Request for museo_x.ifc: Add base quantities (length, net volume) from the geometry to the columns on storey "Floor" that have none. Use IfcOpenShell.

First a look at what the model holds.

```python
import ifcopenshell
import ifcopenshell.util.element
import ifcopenshell.util.unit

model = ifcopenshell.open("museo_x.ifc")
print(model.schema)
for unit_type in ("LENGTHUNIT", "AREAUNIT", "VOLUMEUNIT"):
    print(unit_type, ifcopenshell.util.unit.calculate_unit_scale(model, unit_type))
storey = next(s for s in model.by_type("IfcBuildingStorey") if s.Name == "Floor")
columns = [e for e in ifcopenshell.util.element.get_decomposition(storey) if e.is_a("IfcColumn")]
for e in sorted(columns, key=lambda e: e.id()):
    print(e.id(), e.is_a(), e.Name, list(ifcopenshell.util.element.get_psets(e, qtos_only=True)), sep=" | ")
```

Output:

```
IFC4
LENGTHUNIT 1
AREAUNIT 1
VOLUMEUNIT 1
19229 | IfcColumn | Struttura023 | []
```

```python
import ifcopenshell
import ifcopenshell.api.pset
import ifcopenshell.geom
import ifcopenshell.util.element
import ifcopenshell.util.shape
import ifcopenshell.util.unit

model = ifcopenshell.open("museo_x.ifc")
unit_scale = ifcopenshell.util.unit.calculate_unit_scale(model)
volume_scale = ifcopenshell.util.unit.calculate_unit_scale(model, "VOLUMEUNIT")
settings = ifcopenshell.geom.settings()

storey = next(s for s in model.by_type("IfcBuildingStorey") if s.Name == "Floor")
columns = [e for e in ifcopenshell.util.element.get_decomposition(storey) if e.is_a("IfcColumn")]

for e in sorted(columns, key=lambda e: e.id()):
    if ifcopenshell.util.element.get_psets(e, qtos_only=True, should_inherit=False):
        continue
    # Geometry comes back in metres, in the element's own axes.
    shape = ifcopenshell.geom.create_shape(settings, e)
    values = {
        "Length": ifcopenshell.util.shape.get_z(shape.geometry) / unit_scale,
        "NetVolume": ifcopenshell.util.shape.get_volume(shape.geometry) / volume_scale,
    }
    qto = ifcopenshell.api.pset.add_qto(model, product=e, name="Qto_ColumnBaseQuantities")
    ifcopenshell.api.pset.edit_qto(model, qto=qto, properties=values)
    print(e.id(), {k: round(v, 3) for k, v in values.items()})

model.write("museo_x_rev.ifc")
```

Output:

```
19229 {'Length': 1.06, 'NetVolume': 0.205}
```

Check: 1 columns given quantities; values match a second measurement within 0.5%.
